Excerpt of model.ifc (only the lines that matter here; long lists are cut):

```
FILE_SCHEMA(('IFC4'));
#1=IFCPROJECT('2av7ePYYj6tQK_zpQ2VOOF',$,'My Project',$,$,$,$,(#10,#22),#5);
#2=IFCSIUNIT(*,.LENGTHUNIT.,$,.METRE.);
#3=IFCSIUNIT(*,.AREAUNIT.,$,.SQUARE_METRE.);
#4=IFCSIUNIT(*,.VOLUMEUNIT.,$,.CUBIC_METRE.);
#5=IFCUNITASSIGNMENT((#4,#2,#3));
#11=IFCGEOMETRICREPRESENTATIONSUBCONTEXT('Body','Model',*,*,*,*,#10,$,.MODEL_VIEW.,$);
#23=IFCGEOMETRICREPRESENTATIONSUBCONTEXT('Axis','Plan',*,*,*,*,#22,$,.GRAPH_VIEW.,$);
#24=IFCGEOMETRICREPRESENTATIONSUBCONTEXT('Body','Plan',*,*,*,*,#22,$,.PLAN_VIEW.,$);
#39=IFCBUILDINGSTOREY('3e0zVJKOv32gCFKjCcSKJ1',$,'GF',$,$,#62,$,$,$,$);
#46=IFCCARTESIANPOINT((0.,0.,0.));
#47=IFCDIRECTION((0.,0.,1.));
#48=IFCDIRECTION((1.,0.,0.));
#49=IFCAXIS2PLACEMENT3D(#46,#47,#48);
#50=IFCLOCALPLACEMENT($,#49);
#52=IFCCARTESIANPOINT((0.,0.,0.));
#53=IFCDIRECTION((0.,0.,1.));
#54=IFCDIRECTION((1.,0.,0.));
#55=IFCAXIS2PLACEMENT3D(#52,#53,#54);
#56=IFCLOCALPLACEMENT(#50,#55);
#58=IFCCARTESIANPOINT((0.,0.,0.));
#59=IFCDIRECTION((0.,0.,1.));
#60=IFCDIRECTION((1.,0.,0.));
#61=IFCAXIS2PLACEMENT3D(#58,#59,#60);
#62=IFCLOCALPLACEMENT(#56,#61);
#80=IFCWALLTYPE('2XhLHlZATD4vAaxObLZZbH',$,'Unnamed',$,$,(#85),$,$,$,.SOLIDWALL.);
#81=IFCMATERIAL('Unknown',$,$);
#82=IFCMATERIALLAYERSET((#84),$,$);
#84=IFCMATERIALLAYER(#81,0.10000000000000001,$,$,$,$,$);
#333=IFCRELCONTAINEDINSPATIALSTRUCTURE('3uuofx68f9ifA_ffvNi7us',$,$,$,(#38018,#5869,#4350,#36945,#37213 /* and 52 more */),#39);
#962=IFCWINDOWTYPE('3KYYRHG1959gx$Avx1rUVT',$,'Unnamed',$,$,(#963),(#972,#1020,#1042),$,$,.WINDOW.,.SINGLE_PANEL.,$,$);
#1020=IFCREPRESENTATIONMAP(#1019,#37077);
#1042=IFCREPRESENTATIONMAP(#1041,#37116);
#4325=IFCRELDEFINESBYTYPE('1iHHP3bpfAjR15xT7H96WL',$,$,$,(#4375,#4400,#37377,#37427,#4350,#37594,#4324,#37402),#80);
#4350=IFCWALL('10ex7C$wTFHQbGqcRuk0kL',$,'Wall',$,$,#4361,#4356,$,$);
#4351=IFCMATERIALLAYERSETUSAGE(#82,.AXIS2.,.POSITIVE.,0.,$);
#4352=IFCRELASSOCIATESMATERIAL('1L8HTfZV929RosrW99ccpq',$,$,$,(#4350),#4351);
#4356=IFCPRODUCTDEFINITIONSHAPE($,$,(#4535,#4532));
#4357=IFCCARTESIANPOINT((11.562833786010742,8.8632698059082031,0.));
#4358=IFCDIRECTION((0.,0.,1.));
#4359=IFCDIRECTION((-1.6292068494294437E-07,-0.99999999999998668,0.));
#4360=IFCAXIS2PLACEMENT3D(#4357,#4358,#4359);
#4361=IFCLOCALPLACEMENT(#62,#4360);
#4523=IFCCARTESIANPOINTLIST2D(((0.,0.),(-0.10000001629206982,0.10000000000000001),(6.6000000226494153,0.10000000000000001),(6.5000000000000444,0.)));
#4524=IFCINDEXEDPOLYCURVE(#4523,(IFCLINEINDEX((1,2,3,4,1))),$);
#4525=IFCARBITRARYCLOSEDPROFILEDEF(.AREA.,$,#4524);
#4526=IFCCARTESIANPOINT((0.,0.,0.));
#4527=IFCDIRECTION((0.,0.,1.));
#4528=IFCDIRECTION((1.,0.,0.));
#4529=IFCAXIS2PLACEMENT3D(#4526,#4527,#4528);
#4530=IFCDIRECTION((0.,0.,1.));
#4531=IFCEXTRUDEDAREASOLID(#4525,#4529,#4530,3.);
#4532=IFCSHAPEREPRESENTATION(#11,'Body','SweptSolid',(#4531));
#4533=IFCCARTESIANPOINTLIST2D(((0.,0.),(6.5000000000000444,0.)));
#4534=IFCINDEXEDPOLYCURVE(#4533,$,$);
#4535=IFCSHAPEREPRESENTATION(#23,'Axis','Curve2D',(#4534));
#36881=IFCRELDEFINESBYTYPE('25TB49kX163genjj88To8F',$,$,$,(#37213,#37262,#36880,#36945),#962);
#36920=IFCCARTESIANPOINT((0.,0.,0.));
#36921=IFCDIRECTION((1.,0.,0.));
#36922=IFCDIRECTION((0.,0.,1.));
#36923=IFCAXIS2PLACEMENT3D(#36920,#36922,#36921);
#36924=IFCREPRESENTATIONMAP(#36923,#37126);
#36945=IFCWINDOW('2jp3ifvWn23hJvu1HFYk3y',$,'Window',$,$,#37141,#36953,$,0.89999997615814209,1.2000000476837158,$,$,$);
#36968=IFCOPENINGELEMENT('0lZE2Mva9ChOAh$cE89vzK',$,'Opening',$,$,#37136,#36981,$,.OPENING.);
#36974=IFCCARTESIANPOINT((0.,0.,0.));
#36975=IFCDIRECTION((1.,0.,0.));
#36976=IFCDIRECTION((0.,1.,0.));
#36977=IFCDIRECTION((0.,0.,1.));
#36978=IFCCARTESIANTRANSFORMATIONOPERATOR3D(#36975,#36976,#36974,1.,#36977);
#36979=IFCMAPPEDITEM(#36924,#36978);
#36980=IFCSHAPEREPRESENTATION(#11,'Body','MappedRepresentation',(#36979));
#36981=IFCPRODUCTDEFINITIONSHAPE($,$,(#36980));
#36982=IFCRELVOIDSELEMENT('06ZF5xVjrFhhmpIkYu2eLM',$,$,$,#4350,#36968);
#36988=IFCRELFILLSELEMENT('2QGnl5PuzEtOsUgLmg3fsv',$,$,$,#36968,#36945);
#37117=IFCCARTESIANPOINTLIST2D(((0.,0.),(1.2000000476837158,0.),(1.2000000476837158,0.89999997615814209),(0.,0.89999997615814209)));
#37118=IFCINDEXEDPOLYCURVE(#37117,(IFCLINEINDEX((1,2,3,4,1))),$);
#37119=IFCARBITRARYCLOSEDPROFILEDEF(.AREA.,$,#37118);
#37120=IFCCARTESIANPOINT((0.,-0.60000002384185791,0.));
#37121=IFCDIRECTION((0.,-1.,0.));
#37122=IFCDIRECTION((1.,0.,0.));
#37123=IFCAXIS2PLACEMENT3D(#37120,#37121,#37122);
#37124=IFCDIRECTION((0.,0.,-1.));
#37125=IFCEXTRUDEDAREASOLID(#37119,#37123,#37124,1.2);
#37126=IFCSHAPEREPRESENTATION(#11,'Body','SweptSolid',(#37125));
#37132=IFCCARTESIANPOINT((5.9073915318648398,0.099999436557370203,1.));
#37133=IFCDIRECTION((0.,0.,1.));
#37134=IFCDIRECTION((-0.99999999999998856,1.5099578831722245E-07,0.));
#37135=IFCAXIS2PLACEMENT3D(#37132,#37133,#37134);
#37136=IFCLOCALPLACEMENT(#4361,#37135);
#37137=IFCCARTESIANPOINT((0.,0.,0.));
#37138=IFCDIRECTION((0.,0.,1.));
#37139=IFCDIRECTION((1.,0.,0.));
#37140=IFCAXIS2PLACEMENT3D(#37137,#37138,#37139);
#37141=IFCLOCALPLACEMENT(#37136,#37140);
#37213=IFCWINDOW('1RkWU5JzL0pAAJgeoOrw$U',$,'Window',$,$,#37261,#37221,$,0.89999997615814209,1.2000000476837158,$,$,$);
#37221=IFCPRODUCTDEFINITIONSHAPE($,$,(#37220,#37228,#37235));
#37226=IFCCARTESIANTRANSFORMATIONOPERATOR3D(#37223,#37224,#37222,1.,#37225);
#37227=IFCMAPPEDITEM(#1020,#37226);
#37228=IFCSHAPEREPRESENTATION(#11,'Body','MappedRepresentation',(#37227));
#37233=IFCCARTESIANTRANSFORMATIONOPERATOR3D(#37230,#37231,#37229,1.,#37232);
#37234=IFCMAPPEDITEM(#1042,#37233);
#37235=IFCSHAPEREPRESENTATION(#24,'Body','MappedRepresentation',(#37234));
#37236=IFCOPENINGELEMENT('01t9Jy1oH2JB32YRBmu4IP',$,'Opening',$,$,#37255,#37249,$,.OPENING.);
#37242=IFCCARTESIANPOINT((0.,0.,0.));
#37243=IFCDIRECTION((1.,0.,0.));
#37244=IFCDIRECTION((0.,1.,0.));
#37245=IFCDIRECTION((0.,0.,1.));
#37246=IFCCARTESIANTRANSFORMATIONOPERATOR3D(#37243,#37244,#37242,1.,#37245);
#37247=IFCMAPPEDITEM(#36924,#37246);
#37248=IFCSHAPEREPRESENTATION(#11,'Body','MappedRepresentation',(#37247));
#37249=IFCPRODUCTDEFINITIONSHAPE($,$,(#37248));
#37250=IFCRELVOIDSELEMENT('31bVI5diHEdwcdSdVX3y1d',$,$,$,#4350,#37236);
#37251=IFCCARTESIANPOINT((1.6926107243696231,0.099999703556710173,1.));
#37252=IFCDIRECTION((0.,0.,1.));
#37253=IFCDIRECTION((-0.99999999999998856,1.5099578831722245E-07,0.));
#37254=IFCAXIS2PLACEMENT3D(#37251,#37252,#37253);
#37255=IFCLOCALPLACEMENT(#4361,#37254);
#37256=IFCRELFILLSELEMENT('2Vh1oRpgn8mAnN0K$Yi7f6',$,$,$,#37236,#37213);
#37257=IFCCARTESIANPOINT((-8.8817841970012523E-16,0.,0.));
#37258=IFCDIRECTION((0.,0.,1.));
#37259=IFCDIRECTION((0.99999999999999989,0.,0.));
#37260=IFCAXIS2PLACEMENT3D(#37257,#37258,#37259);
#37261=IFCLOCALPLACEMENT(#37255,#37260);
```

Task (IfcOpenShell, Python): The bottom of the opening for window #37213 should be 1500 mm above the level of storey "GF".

```python
import numpy as np
import ifcopenshell
import ifcopenshell.api.geometry
import ifcopenshell.geom
import ifcopenshell.util.element
import ifcopenshell.util.placement
import ifcopenshell.util.shape
import ifcopenshell.util.unit

model = ifcopenshell.open("model.ifc")
unit_scale = ifcopenshell.util.unit.calculate_unit_scale(model)

window = model.by_guid("1RkWU5JzL0pAAJgeoOrw$U")
opening = window.FillsVoids[0].RelatingOpeningElement
storey = ifcopenshell.util.element.get_container(window, ifc_class="IfcBuildingStorey")
level = ifcopenshell.util.placement.get_local_placement(storey.ObjectPlacement)[2, 3]

# The opening's origin need not be at the sill, so measure its lowest point.
shape = ifcopenshell.geom.create_shape(ifcopenshell.geom.settings(), opening)
bottom = ifcopenshell.util.shape.get_shape_bottom_elevation(shape, shape.geometry) / unit_scale
dz = level + 1.5 / unit_scale - bottom

shift = np.array([0.0, 0.0, dz])
# The window is placed relative to its opening, so it follows when the opening moves.
matrix = ifcopenshell.util.placement.get_local_placement(opening.ObjectPlacement)
matrix[:3, 3] += shift
ifcopenshell.api.geometry.edit_object_placement(
    model, product=opening, matrix=matrix, is_si=False, should_transform_children=True
)

print(f"moved by {dz * unit_scale:+.3f} m")

model.write("model_v2.ifc")
```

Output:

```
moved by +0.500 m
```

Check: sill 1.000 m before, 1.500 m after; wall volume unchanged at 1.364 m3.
